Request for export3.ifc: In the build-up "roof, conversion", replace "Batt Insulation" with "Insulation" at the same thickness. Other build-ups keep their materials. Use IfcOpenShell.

First a look at what the model holds.

```python
import ifcopenshell
import ifcopenshell.util.element

model = ifcopenshell.open("export3.ifc")
print(model.schema)
for layer_set in model.by_type("IfcMaterialLayerSet"):
    if layer_set.LayerSetName == "roof, conversion":
        for layer in layer_set.MaterialLayers:
            print(layer.id(), layer.Material and layer.Material.Name, layer.LayerThickness, sep=" | ")
        print(len(ifcopenshell.util.element.get_elements_by_material(model, layer_set)), "elements and types use it")
print(sorted(m.Name for m in model.by_type("IfcMaterial") if m.Name)[:60])
```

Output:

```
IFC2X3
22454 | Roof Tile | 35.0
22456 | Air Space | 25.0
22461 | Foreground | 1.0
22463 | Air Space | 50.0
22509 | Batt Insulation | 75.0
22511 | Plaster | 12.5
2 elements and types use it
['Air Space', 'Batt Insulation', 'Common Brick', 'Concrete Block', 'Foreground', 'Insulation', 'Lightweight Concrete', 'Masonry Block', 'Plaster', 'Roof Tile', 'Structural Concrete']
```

```python
import ifcopenshell
import ifcopenshell.api.material

model = ifcopenshell.open("export3.ifc")

layer_set = next(s for s in model.by_type("IfcMaterialLayerSet") if s.LayerSetName == "roof, conversion")
layer = next(l for l in layer_set.MaterialLayers if l.Material and l.Material.Name == "Batt Insulation")
material = next(m for m in model.by_type("IfcMaterial") if m.Name == "Insulation")

# Point this one layer at the other material; renaming the old one would change it everywhere.
ifcopenshell.api.material.edit_layer(model, layer=layer, attributes={}, material=material)

print([l.Material.Name if l.Material else None for l in layer_set.MaterialLayers])

model.write("export3-out.ifc")
```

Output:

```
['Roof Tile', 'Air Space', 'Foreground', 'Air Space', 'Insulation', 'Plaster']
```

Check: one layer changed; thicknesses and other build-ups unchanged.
